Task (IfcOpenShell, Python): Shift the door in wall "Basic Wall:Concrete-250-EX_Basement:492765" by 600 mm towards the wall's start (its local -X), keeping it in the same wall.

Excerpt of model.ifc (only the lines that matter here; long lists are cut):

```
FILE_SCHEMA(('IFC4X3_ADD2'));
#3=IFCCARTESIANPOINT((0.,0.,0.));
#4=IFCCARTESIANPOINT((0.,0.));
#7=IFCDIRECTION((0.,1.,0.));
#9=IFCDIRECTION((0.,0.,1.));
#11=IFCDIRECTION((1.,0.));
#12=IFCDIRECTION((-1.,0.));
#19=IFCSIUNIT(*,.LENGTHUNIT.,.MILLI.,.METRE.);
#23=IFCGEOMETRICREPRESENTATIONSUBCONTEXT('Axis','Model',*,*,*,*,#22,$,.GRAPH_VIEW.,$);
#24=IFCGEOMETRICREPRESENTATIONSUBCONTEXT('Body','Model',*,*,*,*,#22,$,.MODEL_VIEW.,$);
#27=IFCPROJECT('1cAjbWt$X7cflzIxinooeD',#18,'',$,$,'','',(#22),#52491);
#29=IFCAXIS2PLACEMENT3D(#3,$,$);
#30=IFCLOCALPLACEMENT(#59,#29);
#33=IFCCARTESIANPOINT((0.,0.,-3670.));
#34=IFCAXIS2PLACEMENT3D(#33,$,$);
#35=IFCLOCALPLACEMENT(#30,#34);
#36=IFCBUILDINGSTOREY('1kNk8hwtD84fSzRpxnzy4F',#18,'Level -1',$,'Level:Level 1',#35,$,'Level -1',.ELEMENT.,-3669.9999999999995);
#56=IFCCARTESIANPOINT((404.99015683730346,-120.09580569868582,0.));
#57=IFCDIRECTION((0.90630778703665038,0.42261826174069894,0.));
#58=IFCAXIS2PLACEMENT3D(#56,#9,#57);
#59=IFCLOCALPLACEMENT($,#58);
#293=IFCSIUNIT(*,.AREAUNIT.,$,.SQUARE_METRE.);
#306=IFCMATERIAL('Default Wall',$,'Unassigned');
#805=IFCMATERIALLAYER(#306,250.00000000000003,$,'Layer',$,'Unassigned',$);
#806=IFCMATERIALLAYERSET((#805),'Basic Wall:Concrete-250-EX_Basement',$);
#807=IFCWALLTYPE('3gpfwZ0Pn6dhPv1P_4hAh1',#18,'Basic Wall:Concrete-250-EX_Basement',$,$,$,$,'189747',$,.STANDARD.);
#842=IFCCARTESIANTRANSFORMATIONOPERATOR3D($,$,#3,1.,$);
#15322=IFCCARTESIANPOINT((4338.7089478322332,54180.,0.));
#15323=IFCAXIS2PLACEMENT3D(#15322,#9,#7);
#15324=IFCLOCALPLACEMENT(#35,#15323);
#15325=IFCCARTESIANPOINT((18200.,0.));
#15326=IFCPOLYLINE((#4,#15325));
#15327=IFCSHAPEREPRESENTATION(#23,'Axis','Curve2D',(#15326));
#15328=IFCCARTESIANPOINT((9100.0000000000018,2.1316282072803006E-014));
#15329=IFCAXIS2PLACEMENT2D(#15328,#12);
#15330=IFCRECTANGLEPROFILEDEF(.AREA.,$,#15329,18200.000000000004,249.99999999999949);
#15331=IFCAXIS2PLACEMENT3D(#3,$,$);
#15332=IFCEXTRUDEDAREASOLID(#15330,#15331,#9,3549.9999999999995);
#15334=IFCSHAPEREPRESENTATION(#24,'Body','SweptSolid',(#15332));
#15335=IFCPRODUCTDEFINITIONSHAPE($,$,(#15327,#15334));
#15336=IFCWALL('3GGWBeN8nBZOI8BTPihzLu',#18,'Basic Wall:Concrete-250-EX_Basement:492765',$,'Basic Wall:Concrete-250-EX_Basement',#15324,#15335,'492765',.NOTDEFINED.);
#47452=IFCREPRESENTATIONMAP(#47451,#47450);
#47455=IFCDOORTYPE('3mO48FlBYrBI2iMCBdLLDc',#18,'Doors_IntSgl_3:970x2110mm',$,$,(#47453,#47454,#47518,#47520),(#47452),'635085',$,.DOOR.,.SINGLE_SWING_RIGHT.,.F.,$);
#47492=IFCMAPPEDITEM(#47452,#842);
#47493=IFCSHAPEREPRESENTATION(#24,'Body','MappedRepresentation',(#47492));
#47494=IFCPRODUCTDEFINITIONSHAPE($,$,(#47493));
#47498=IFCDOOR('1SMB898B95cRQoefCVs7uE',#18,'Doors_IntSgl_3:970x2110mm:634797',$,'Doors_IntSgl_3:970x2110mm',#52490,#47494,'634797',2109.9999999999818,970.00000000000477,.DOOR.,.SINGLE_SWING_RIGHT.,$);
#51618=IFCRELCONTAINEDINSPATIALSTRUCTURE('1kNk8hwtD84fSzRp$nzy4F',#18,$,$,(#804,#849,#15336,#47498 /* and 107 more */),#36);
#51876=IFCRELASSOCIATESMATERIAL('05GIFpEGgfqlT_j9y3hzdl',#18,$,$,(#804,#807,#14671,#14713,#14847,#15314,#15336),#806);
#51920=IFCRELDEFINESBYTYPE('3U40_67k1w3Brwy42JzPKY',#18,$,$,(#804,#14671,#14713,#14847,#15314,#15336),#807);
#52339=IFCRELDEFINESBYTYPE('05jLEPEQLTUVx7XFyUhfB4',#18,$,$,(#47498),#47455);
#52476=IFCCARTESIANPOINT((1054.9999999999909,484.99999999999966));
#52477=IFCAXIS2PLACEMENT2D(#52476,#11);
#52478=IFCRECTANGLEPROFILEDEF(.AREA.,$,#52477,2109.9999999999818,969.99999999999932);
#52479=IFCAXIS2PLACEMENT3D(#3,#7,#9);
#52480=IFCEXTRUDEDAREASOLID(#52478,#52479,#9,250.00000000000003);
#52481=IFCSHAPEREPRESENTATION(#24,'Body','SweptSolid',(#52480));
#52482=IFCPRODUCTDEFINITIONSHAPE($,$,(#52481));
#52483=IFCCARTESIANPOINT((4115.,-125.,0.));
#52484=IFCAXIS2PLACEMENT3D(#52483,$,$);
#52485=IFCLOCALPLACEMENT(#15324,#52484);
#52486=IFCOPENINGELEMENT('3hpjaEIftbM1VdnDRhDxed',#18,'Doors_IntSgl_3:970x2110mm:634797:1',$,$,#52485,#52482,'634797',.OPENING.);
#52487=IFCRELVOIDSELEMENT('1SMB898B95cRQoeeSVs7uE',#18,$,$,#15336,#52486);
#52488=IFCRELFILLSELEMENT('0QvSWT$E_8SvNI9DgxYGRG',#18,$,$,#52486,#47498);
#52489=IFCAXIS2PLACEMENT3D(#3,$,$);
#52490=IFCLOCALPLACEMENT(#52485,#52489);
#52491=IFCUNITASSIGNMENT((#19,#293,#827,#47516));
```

```python
import ifcopenshell
import ifcopenshell.api.geometry
import ifcopenshell.util.placement
import ifcopenshell.util.unit

model = ifcopenshell.open("model.ifc")
unit_scale = ifcopenshell.util.unit.calculate_unit_scale(model)

door = model.by_id(47498)
opening = door.FillsVoids[0].RelatingOpeningElement
wall = opening.VoidsElements[0].RelatingBuildingElement

wall_matrix = ifcopenshell.util.placement.get_local_placement(wall.ObjectPlacement)
shift = wall_matrix[:3, 0] * -0.6 / unit_scale
before = ifcopenshell.util.placement.get_local_placement(door.ObjectPlacement)[:3, 3].copy()

# The door is placed relative to its opening, so it follows when the opening moves.
matrix = ifcopenshell.util.placement.get_local_placement(opening.ObjectPlacement)
matrix[:3, 3] += shift
ifcopenshell.api.geometry.edit_object_placement(
    model, product=opening, matrix=matrix, is_si=False, should_transform_children=True
)

after = ifcopenshell.util.placement.get_local_placement(door.ObjectPlacement)[:3, 3]
print("door moved by", (after - before).round(3) + 0.0)

model.write("model_v2.ifc")
```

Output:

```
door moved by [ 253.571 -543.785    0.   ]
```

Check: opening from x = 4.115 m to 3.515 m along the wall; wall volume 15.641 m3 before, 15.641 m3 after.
